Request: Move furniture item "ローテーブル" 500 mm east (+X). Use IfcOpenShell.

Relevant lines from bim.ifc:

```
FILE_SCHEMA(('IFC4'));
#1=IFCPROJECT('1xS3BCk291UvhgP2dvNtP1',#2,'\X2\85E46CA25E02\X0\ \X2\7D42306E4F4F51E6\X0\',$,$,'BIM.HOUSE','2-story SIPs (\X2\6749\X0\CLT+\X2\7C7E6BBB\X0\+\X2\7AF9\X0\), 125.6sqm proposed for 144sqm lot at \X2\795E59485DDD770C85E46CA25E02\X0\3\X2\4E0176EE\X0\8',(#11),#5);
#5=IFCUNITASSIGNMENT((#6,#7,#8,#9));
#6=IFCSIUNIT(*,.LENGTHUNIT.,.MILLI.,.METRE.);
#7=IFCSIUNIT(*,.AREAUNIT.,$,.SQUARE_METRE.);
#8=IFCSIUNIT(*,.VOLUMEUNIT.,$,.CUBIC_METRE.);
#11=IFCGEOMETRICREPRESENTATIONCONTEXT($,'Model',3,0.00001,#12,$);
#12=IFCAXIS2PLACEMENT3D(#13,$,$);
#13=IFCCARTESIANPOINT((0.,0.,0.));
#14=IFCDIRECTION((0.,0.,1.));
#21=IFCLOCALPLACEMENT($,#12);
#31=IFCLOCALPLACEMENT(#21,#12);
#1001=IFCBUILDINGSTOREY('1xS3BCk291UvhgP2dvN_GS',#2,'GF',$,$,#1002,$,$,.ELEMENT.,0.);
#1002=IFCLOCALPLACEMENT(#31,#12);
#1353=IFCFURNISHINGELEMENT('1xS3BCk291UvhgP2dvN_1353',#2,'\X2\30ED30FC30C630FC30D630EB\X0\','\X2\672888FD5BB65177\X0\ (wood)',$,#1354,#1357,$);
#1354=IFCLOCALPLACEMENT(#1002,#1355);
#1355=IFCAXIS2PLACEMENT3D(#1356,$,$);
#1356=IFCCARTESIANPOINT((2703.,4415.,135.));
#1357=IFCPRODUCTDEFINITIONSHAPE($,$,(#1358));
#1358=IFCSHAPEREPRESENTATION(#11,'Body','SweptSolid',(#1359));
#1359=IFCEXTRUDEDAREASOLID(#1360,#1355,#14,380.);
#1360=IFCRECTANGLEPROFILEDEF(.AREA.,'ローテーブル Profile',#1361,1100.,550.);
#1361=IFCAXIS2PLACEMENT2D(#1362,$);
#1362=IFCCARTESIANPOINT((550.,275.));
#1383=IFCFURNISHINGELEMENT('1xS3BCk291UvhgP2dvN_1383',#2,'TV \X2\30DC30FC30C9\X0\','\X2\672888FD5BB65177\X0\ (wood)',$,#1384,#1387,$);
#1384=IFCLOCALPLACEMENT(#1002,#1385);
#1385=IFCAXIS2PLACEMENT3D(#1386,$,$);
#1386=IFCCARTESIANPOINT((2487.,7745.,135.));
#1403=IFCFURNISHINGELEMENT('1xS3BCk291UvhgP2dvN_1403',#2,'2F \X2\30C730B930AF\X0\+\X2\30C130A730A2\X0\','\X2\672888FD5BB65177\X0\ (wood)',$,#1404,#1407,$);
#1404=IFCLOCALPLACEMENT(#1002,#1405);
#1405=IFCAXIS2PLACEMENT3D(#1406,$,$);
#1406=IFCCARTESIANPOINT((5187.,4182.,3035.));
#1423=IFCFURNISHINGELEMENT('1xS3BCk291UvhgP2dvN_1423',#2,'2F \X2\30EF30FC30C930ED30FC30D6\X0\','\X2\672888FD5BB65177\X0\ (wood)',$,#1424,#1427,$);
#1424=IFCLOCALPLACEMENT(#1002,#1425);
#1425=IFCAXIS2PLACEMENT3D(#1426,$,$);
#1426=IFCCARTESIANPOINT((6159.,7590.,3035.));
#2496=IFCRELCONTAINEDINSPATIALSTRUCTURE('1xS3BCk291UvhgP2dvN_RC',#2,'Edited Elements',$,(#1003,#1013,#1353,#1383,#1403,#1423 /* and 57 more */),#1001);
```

```python
import ifcopenshell
import ifcopenshell.api.geometry
import ifcopenshell.util.placement
import ifcopenshell.util.unit

model = ifcopenshell.open("bim.ifc")
unit_scale = ifcopenshell.util.unit.calculate_unit_scale(model)

item = model.by_id(1353)
matrix = ifcopenshell.util.placement.get_local_placement(item.ObjectPlacement)
matrix[0, 3] += 0.5 / unit_scale
ifcopenshell.api.geometry.edit_object_placement(model, product=item, matrix=matrix, is_si=False)

print(ifcopenshell.util.placement.get_local_placement(item.ObjectPlacement).round(3) + 0.0)

model.write("bim_edited.ifc")
```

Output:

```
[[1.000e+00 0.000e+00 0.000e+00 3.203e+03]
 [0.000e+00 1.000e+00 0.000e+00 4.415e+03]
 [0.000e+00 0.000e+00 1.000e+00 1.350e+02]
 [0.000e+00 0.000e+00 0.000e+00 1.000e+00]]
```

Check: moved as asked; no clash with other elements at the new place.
